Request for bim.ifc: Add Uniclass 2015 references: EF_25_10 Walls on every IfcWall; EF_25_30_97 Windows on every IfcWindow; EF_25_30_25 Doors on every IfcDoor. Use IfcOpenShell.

First a look at what the model holds.

```python
import ifcopenshell

model = ifcopenshell.open("bim.ifc")
print(model.schema)
print("classifications:", [c.Name for c in model.by_type("IfcClassification")])
for ifc_class in ("IfcDoor", "IfcRoof", "IfcStair", "IfcWall", "IfcWindow"):
    print(ifc_class, len(model.by_type(ifc_class)))
```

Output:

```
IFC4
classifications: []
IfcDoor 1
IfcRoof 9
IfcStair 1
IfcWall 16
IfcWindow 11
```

```python
import ifcopenshell
import ifcopenshell.api.classification

model = ifcopenshell.open("bim.ifc")

system = ifcopenshell.api.classification.add_classification(model, classification="Uniclass 2015")

codes = {
    "IfcWall": ("EF_25_10", "Walls"),
    "IfcWindow": ("EF_25_30_97", "Windows"),
    "IfcDoor": ("EF_25_30_25", "Doors"),
}
for ifc_class, (code, name) in codes.items():
    products = model.by_type(ifc_class)
    ifcopenshell.api.classification.add_reference(
        model, products=products, classification=system, identification=code, name=name
    )
    print(code, len(products))

model.write("bim-out.ifc")
```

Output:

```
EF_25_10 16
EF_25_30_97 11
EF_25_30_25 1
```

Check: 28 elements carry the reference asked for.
